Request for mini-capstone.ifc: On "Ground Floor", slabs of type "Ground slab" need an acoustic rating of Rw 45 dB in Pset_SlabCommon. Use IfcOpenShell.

First a look at what the model holds.

```python
import ifcopenshell
import ifcopenshell.util.element

model = ifcopenshell.open("mini-capstone.ifc")
print(model.schema)
storey = next(s for s in model.by_type("IfcBuildingStorey") if s.Name == "Ground Floor")
slabs = [e for e in ifcopenshell.util.element.get_decomposition(storey) if e.is_a("IfcSlab")]
seen = {}
for e in slabs:
    element_type = ifcopenshell.util.element.get_type(e)
    key = (element_type.Name if element_type != e and element_type else None, ifcopenshell.util.element.get_pset(e, "Pset_SlabCommon", "AcousticRating"))
    seen[key] = seen.get(key, 0) + 1
for (name, value), count in sorted(seen.items(), key=str):
    print(count, "x", name, "|", value)
```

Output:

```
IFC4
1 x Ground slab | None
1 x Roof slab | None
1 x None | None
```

```python
import ifcopenshell
import ifcopenshell.api.pset
import ifcopenshell.util.element

model = ifcopenshell.open("mini-capstone.ifc")

storey = next(s for s in model.by_type("IfcBuildingStorey") if s.Name == "Ground Floor")
slabs = [e for e in ifcopenshell.util.element.get_decomposition(storey) if e.is_a("IfcSlab")]

count = 0
for e in slabs:
    element_type = ifcopenshell.util.element.get_type(e)
    if element_type in (None, e) or element_type.Name != "Ground slab":
        continue
    # add_pset returns the element's existing set when there is one.
    pset = ifcopenshell.api.pset.add_pset(model, product=e, name="Pset_SlabCommon")
    ifcopenshell.api.pset.edit_pset(model, pset=pset, properties={"AcousticRating": "Rw 45 dB"})
    count += 1

print(count, "slabs updated")

model.write("mini-capstone_updated.ifc")
```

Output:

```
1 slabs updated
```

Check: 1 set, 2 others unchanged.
